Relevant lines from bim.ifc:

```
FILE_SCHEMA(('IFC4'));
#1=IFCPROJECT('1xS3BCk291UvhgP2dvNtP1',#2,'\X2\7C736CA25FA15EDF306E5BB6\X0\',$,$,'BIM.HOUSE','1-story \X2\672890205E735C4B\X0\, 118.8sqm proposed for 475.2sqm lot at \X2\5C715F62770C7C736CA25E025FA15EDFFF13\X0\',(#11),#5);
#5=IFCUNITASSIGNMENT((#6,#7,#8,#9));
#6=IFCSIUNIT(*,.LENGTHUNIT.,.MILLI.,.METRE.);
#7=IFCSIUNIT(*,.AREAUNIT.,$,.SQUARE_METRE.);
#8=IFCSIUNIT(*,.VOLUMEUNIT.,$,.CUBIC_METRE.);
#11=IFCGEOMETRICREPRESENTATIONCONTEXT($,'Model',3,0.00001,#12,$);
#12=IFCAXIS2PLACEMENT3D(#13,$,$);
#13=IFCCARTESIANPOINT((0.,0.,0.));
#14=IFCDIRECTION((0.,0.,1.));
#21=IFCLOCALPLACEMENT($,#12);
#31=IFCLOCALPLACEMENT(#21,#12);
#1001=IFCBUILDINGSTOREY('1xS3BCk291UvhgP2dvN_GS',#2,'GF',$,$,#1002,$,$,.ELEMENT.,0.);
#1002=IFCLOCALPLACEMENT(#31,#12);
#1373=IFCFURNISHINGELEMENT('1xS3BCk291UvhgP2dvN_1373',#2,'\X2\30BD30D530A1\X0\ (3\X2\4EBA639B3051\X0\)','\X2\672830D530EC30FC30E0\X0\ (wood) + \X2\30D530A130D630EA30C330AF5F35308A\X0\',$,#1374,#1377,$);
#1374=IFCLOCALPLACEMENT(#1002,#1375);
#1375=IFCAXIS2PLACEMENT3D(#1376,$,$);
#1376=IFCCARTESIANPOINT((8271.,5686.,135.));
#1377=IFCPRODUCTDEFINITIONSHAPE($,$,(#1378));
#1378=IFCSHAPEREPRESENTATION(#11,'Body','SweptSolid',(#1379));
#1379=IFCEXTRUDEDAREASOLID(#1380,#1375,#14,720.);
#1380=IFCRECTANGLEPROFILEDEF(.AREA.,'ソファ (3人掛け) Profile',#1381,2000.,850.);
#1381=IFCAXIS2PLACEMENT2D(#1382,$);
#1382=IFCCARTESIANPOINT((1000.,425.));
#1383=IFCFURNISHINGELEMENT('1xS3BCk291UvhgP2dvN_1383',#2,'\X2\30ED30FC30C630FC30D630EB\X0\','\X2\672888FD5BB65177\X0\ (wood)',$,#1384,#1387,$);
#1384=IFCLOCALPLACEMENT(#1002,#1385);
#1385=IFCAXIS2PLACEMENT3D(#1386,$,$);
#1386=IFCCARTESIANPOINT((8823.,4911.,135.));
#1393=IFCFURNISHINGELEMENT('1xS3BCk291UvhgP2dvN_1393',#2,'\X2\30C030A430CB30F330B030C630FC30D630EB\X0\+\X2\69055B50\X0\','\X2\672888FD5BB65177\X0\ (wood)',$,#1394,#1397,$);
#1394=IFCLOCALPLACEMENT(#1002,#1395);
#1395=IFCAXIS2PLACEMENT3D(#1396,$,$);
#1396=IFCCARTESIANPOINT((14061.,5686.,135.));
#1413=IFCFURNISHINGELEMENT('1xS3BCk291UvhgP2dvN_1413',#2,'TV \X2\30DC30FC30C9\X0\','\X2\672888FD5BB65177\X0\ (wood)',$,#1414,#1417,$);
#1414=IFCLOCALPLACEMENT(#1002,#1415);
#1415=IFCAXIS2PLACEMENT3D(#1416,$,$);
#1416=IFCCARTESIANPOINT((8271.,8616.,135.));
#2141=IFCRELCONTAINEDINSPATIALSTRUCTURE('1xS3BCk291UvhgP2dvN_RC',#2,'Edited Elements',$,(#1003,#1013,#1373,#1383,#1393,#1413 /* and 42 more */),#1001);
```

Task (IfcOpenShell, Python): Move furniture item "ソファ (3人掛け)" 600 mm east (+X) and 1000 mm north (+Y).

```python
import ifcopenshell
import ifcopenshell.api.geometry
import ifcopenshell.util.placement

model = ifcopenshell.open("bim.ifc")

item = model.by_id(1373)
matrix = ifcopenshell.util.placement.get_local_placement(item.ObjectPlacement)
matrix[0, 3] += 600.0
matrix[1, 3] += 1000.0
ifcopenshell.api.geometry.edit_object_placement(model, product=item, matrix=matrix, is_si=False)

print(ifcopenshell.util.placement.get_local_placement(item.ObjectPlacement).round(3) + 0.0)

model.write("bim-out.ifc")
```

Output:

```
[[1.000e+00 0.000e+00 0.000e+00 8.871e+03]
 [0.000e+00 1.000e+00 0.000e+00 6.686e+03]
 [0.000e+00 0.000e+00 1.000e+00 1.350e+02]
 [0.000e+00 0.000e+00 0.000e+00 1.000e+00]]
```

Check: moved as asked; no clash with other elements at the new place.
